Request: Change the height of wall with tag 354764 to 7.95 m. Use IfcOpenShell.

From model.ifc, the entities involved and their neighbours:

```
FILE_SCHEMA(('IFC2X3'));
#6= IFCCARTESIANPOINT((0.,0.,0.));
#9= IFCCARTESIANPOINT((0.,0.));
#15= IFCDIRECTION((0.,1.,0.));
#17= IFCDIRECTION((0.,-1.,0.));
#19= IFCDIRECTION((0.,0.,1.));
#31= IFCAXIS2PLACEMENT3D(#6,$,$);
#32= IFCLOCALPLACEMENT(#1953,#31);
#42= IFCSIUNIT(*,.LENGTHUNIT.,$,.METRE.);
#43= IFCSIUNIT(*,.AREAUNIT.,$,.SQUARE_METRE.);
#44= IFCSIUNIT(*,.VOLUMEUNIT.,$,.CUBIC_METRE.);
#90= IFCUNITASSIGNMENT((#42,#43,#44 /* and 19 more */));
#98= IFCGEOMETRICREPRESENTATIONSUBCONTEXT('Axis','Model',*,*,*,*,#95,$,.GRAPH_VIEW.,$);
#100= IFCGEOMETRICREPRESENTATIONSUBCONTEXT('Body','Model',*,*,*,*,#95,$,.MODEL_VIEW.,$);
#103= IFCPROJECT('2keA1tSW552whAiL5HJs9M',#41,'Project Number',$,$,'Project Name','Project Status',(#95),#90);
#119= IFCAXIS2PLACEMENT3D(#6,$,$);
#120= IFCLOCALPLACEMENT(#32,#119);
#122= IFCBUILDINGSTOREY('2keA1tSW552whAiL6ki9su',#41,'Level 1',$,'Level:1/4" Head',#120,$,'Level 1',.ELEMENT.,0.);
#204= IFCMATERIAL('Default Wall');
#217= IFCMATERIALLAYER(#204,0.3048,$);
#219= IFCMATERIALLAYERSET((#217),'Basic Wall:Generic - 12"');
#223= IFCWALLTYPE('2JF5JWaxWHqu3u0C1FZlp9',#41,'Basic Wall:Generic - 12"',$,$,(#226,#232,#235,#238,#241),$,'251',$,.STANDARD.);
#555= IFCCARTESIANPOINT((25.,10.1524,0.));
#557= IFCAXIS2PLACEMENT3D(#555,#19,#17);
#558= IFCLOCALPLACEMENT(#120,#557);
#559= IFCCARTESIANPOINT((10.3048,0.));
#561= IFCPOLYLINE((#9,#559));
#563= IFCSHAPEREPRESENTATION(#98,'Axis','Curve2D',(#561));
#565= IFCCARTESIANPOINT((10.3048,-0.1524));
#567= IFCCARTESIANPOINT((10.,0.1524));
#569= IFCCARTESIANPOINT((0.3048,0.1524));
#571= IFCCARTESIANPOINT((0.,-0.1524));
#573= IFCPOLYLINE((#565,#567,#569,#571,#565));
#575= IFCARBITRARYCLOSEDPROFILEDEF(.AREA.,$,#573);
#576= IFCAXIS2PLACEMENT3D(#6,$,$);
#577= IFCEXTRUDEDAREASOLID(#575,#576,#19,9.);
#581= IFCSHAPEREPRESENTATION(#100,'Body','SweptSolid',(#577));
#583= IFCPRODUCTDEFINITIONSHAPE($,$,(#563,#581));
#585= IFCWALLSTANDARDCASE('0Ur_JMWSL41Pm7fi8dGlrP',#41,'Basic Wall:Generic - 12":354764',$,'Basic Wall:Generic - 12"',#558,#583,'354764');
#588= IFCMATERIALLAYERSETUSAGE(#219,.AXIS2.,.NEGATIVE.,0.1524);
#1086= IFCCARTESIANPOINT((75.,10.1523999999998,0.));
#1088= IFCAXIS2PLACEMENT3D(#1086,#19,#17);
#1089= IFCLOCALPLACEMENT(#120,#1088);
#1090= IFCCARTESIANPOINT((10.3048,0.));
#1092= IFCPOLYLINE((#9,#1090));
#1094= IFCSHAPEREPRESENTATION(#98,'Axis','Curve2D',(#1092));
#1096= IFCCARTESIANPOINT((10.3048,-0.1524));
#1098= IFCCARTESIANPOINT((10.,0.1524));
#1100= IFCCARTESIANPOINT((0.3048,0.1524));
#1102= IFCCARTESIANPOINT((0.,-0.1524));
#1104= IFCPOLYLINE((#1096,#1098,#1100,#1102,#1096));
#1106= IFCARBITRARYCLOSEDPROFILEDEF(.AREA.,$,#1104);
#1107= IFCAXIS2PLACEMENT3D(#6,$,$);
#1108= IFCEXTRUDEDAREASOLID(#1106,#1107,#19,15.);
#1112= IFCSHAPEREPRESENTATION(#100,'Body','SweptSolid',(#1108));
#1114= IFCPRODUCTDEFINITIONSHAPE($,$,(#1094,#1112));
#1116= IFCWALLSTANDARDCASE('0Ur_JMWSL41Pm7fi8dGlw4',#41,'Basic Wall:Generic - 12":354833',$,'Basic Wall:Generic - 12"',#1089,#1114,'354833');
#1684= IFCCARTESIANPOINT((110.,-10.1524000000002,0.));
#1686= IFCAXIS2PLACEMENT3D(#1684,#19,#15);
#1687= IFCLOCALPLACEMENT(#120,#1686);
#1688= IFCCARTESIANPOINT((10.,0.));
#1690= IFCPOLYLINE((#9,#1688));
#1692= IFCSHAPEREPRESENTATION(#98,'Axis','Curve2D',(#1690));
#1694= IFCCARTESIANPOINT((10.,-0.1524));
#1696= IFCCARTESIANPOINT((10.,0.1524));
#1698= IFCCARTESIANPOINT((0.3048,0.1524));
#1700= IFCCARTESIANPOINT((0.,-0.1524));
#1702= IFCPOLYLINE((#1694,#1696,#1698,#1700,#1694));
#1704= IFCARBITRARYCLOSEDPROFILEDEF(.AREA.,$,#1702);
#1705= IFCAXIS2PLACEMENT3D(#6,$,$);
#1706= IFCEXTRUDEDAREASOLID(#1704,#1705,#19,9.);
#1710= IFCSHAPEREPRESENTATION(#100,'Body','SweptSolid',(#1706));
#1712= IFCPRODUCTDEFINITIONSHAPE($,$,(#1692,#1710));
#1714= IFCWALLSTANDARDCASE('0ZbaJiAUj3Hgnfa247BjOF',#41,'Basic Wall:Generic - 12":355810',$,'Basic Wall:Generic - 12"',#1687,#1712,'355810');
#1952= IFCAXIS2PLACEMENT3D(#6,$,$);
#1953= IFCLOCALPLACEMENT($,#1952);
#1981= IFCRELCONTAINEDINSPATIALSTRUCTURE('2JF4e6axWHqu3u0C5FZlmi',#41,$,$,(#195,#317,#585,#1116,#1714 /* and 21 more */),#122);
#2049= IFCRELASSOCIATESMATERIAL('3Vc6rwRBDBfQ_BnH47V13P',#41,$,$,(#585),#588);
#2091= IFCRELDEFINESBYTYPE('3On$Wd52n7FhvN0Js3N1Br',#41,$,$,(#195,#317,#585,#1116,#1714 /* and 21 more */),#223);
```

```python
import ifcopenshell
import ifcopenshell.geom
import ifcopenshell.util.representation
import ifcopenshell.util.shape

model = ifcopenshell.open("model.ifc")
settings = ifcopenshell.geom.settings()


def volume(element):
    """Net volume in cubic metres, openings subtracted."""
    shape = ifcopenshell.geom.create_shape(settings, element)
    return ifcopenshell.util.shape.get_volume(shape.geometry)


wall = model.by_guid("0Ur_JMWSL41Pm7fi8dGlrP")
before = volume(wall)

body = ifcopenshell.util.representation.get_representation(wall, "Model", "Body")
solid = body.Items[0]
old_height = solid.Depth
solid.Depth = 7.95
after = volume(wall)

print(f"height {old_height:g} -> {solid.Depth:g}, volume {before:.3f} -> {after:.3f} m3")

model.write("model_v2.ifc")
```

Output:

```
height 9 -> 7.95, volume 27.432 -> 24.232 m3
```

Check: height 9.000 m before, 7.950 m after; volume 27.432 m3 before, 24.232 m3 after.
